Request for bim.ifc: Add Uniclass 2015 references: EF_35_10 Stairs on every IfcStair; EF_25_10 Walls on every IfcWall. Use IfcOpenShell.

First a look at what the model holds.

```python
import ifcopenshell

model = ifcopenshell.open("bim.ifc")
print(model.schema)
print("classifications:", [c.Name for c in model.by_type("IfcClassification")])
for ifc_class in ("IfcDoor", "IfcRoof", "IfcStair", "IfcWall", "IfcWindow"):
    print(ifc_class, len(model.by_type(ifc_class)))
```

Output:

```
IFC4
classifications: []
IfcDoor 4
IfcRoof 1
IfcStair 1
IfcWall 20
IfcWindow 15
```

```python
import ifcopenshell
import ifcopenshell.api.classification

model = ifcopenshell.open("bim.ifc")

system = ifcopenshell.api.classification.add_classification(model, classification="Uniclass 2015")

codes = {
    "IfcStair": ("EF_35_10", "Stairs"),
    "IfcWall": ("EF_25_10", "Walls"),
}
for ifc_class, (code, name) in codes.items():
    products = model.by_type(ifc_class)
    ifcopenshell.api.classification.add_reference(
        model, products=products, classification=system, identification=code, name=name
    )
    print(code, len(products))

model.write("bim-out.ifc")
```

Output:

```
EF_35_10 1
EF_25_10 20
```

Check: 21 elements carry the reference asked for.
